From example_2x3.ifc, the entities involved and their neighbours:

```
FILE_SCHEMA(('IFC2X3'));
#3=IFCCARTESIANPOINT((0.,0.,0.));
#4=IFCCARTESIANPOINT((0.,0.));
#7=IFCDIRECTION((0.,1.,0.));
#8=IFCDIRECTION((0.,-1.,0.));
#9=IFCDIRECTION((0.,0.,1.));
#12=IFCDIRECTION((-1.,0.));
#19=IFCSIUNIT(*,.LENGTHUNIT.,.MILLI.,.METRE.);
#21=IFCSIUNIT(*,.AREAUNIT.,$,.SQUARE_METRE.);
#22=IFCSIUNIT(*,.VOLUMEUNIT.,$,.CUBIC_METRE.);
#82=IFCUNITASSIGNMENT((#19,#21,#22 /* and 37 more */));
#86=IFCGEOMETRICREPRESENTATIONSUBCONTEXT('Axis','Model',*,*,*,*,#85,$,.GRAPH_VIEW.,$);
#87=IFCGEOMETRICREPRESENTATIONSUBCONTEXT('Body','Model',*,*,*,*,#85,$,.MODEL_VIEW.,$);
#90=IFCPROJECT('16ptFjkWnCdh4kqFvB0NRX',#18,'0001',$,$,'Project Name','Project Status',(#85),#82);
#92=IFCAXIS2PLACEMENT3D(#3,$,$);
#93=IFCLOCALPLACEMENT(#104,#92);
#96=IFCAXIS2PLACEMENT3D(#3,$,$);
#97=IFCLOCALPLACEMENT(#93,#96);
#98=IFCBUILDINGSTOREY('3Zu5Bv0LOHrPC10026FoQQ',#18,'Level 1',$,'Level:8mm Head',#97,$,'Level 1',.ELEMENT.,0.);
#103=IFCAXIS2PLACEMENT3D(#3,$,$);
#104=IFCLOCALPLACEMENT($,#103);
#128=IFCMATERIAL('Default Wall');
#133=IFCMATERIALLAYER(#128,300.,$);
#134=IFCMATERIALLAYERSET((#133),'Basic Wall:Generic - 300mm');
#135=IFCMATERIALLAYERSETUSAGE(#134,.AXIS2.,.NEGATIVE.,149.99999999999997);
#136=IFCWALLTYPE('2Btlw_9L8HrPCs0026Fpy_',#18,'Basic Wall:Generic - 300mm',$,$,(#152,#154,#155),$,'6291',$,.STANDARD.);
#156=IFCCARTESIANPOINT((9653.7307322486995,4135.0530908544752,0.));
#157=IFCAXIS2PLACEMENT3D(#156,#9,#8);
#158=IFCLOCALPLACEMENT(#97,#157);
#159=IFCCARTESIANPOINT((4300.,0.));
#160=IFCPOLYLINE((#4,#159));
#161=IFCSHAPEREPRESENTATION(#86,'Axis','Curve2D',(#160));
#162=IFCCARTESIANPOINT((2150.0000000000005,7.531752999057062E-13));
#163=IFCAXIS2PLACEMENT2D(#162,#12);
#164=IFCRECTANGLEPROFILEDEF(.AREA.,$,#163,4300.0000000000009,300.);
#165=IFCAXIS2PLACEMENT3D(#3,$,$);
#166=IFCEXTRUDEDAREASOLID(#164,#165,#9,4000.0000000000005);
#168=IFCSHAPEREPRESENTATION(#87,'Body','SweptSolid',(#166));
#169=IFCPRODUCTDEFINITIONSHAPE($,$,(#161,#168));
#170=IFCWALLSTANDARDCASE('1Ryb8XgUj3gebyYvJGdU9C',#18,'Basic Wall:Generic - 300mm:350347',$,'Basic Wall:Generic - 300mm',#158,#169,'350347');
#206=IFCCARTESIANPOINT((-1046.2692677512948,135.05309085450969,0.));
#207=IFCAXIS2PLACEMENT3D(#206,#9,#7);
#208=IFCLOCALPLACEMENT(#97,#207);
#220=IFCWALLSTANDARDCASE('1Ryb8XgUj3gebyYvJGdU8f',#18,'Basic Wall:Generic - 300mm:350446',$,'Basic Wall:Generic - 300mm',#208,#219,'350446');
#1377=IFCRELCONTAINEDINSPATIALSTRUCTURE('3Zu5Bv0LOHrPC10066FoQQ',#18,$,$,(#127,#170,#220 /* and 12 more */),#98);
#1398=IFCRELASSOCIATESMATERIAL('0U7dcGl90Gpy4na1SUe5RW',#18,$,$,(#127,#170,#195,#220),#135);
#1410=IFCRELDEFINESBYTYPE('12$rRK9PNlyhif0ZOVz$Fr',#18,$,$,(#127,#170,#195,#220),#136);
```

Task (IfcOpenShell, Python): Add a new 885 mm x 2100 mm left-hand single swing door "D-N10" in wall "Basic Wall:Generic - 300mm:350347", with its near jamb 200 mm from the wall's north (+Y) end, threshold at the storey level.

```python
import numpy as np
import ifcopenshell
import ifcopenshell.api.feature
import ifcopenshell.api.geometry
import ifcopenshell.api.root
import ifcopenshell.api.spatial
import ifcopenshell.api.type
import ifcopenshell.geom
import ifcopenshell.util.element
import ifcopenshell.util.placement
import ifcopenshell.util.representation
import ifcopenshell.util.shape
import ifcopenshell.util.unit

model = ifcopenshell.open("example_2x3.ifc")
unit_scale = ifcopenshell.util.unit.calculate_unit_scale(model)
settings = ifcopenshell.geom.settings()


def volume(element):
    """Net volume in cubic metres, openings subtracted."""
    shape = ifcopenshell.geom.create_shape(settings, element)
    return ifcopenshell.util.shape.get_volume(shape.geometry)


wall = model.by_guid("1Ryb8XgUj3gebyYvJGdU9C")
storey = ifcopenshell.util.element.get_container(wall, ifc_class="IfcBuildingStorey")
context = ifcopenshell.util.representation.get_context(model, "Model", "Body", "MODEL_VIEW")
before = volume(wall)

width, height, from_end, sill = 0.885, 2.1, 0.2, 0.0  # metres

# The wall runs along its own X axis, and the end named is its -X end.
wall_shape = ifcopenshell.geom.create_shape(settings, wall)
x, y, z = ifcopenshell.util.shape.get_vertices(wall_shape.geometry).T
start = x.min() + from_end
face, thickness = float(y.min()), float(y.max() - y.min())
wall_matrix = ifcopenshell.util.placement.get_local_placement(wall.ObjectPlacement)
level = ifcopenshell.util.placement.get_local_placement(storey.ObjectPlacement)[2, 3]


def in_wall(x, y):
    """Placement at x, y metres in the wall's axes, at sill height."""
    matrix = wall_matrix.copy()
    matrix[:, 3] = wall_matrix @ np.array([x / unit_scale, y / unit_scale, 0.0, 1.0])
    matrix[2, 3] = level + sill / unit_scale
    return matrix


# Opening: a box that overshoots both wall faces by 50 mm.
opening = ifcopenshell.api.root.create_entity(model, ifc_class="IfcOpeningElement")
box = ifcopenshell.api.geometry.add_wall_representation(
    model, context=context, length=width, height=height, thickness=thickness + 0.1
)
ifcopenshell.api.geometry.assign_representation(model, product=opening, representation=box)
ifcopenshell.api.geometry.edit_object_placement(model, product=opening, matrix=in_wall(start, face - 0.05), is_si=False)
ifcopenshell.api.feature.add_feature(model, feature=opening, element=wall)

door = ifcopenshell.api.root.create_entity(model, ifc_class="IfcDoor", name="D-N10")
door.OverallWidth, door.OverallHeight = width / unit_scale, height / unit_scale
body = ifcopenshell.api.geometry.add_door_representation(
    model,
    context=context,
    overall_width=door.OverallWidth,
    overall_height=door.OverallHeight,
    operation_type="SINGLE_SWING_LEFT",
    lining_properties={"LiningDepth": thickness / unit_scale, "ThresholdDepth": thickness / unit_scale},
)
ifcopenshell.api.geometry.assign_representation(model, product=door, representation=body)
ifcopenshell.api.spatial.assign_container(model, products=[door], relating_structure=storey)
fills = ifcopenshell.api.feature.add_filling(model, opening=opening, element=door)
fills.OwnerHistory = door.OwnerHistory  # required in IFC2X3

# IFC2X3 keeps the operation on the door style.
style = ifcopenshell.api.root.create_entity(model, ifc_class="IfcDoorStyle", name="D-N10")
style.OperationType, style.ConstructionType = "SINGLE_SWING_LEFT", "NOTDEFINED"
style.ParameterTakesPrecedence = style.Sizeable = False
ifcopenshell.api.type.assign_type(model, related_objects=[door], relating_type=style)

# The lining spans the wall, so the door starts at the wall face.
ifcopenshell.api.geometry.edit_object_placement(model, product=door, matrix=in_wall(start, face), is_si=False)

after = volume(wall)

print(f"wall volume {before:.3f} -> {after:.3f} m3")

model.write("example_2x3_edited.ifc")
```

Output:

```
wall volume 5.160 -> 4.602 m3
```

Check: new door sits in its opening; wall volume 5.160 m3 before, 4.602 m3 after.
